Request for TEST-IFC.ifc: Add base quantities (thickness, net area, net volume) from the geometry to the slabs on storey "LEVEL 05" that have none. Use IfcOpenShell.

First a look at what the model holds.

```python
import ifcopenshell
import ifcopenshell.util.element
import ifcopenshell.util.unit

model = ifcopenshell.open("TEST-IFC.ifc")
print(model.schema)
for unit_type in ("LENGTHUNIT", "AREAUNIT", "VOLUMEUNIT"):
    print(unit_type, ifcopenshell.util.unit.calculate_unit_scale(model, unit_type))
storey = next(s for s in model.by_type("IfcBuildingStorey") if s.Name == "LEVEL 05")
slabs = [e for e in ifcopenshell.util.element.get_decomposition(storey) if e.is_a("IfcSlab")]
for e in sorted(slabs, key=lambda e: e.id()):
    print(e.id(), e.is_a(), e.Name, list(ifcopenshell.util.element.get_psets(e, qtos_only=True)), sep=" | ")
```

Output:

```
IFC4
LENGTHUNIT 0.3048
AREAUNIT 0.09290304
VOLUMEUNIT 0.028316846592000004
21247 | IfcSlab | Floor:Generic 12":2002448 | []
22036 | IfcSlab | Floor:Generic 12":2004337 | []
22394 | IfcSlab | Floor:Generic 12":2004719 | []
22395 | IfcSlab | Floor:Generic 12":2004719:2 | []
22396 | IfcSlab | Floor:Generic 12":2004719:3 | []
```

```python
import ifcopenshell
import ifcopenshell.api.pset
import ifcopenshell.geom
import ifcopenshell.util.element
import ifcopenshell.util.shape
import ifcopenshell.util.unit

model = ifcopenshell.open("TEST-IFC.ifc")
unit_scale = ifcopenshell.util.unit.calculate_unit_scale(model)
area_scale = ifcopenshell.util.unit.calculate_unit_scale(model, "AREAUNIT")
volume_scale = ifcopenshell.util.unit.calculate_unit_scale(model, "VOLUMEUNIT")
settings = ifcopenshell.geom.settings()

storey = next(s for s in model.by_type("IfcBuildingStorey") if s.Name == "LEVEL 05")
slabs = [e for e in ifcopenshell.util.element.get_decomposition(storey) if e.is_a("IfcSlab")]

for e in sorted(slabs, key=lambda e: e.id()):
    if ifcopenshell.util.element.get_psets(e, qtos_only=True, should_inherit=False):
        continue
    # Geometry comes back in metres, in the element's own axes.
    shape = ifcopenshell.geom.create_shape(settings, e)
    values = {
        "Width": ifcopenshell.util.shape.get_z(shape.geometry) / unit_scale,
        "NetArea": ifcopenshell.util.shape.get_footprint_area(shape.geometry) / area_scale,
        "NetVolume": ifcopenshell.util.shape.get_volume(shape.geometry) / volume_scale,
    }
    qto = ifcopenshell.api.pset.add_qto(model, product=e, name="Qto_SlabBaseQuantities")
    ifcopenshell.api.pset.edit_qto(model, qto=qto, properties=values)
    print(e.id(), {k: round(v, 3) for k, v in values.items()})

model.write("TEST-IFC_v2.ifc")
```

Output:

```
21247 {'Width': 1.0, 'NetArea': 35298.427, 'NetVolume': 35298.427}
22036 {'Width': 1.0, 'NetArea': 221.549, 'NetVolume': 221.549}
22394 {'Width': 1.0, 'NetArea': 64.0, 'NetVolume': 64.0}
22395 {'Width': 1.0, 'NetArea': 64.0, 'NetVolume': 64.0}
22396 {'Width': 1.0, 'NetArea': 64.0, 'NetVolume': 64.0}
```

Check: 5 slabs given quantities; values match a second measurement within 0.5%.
